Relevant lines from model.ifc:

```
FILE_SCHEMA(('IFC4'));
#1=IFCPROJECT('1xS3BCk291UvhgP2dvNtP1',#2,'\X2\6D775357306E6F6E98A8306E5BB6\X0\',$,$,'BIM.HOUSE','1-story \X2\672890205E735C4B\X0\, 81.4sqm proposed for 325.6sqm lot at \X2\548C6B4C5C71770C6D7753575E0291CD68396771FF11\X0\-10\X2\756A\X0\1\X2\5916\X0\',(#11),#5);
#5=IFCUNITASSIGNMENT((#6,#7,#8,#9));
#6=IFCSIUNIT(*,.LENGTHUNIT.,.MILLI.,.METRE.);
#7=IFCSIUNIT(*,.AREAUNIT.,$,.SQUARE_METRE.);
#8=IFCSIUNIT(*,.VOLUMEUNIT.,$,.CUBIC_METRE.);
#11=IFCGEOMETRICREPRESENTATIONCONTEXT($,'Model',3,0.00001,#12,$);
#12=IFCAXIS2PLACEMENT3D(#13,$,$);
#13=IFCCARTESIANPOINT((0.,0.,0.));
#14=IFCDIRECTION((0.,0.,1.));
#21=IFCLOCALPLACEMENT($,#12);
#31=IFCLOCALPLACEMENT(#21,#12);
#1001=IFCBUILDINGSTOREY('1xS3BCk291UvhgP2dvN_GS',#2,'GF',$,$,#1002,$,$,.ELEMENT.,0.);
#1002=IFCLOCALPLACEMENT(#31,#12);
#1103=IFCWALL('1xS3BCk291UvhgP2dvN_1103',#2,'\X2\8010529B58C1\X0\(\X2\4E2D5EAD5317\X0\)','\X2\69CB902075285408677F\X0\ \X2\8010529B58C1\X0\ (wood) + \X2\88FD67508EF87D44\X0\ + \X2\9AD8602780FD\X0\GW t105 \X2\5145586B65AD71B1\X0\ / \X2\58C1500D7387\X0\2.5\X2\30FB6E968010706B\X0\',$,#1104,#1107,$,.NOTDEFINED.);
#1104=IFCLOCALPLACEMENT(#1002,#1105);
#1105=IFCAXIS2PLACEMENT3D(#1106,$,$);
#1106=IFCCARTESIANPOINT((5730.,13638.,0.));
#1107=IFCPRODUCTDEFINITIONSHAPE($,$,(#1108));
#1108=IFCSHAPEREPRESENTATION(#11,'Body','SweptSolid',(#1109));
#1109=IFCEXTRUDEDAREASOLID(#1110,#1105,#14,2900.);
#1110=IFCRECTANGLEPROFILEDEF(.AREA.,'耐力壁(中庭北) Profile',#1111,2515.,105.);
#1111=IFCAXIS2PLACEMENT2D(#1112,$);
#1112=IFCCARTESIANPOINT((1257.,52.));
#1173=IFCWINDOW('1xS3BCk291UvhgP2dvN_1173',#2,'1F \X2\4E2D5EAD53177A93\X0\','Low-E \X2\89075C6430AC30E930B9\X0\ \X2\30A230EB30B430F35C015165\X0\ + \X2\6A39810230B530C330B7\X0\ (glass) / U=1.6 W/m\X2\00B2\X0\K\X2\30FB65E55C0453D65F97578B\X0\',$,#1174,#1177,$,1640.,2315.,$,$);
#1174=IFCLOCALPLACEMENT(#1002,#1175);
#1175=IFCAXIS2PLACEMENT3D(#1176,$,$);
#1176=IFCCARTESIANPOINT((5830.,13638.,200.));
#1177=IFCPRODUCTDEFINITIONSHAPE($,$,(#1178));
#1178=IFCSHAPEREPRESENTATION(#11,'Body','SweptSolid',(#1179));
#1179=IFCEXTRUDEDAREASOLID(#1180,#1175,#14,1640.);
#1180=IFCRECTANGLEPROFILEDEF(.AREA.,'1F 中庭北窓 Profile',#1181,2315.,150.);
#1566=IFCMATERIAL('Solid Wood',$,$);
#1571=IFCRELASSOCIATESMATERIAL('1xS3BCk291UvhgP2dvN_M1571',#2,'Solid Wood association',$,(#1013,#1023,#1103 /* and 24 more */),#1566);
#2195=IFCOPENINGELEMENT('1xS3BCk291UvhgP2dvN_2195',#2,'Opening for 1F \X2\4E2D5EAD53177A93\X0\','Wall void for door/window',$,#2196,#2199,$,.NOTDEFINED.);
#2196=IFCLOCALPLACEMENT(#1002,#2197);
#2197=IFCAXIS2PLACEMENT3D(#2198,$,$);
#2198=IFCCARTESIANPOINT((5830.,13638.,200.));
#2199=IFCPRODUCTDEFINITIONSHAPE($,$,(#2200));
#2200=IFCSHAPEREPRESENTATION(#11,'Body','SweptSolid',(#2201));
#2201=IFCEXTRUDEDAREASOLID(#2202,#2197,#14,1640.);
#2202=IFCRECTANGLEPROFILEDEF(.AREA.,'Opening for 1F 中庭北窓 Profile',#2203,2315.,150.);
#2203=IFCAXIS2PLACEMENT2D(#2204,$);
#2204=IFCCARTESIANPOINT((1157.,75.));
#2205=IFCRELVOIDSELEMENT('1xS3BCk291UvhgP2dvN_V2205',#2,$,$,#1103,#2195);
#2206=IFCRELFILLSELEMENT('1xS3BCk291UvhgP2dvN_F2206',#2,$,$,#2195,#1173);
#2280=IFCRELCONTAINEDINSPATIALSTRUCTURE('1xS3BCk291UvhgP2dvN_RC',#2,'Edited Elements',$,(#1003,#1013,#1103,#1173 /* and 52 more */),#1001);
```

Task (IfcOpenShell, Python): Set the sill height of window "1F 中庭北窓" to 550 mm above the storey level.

```python
import numpy as np
import ifcopenshell
import ifcopenshell.api.geometry
import ifcopenshell.geom
import ifcopenshell.util.element
import ifcopenshell.util.placement
import ifcopenshell.util.shape
import ifcopenshell.util.unit

model = ifcopenshell.open("model.ifc")
unit_scale = ifcopenshell.util.unit.calculate_unit_scale(model)

window = model.by_guid("1xS3BCk291UvhgP2dvN_1173")
opening = window.FillsVoids[0].RelatingOpeningElement
storey = ifcopenshell.util.element.get_container(window, ifc_class="IfcBuildingStorey")
level = ifcopenshell.util.placement.get_local_placement(storey.ObjectPlacement)[2, 3]

# The opening's origin need not be at the sill, so measure its lowest point.
shape = ifcopenshell.geom.create_shape(ifcopenshell.geom.settings(), opening)
bottom = ifcopenshell.util.shape.get_shape_bottom_elevation(shape, shape.geometry) / unit_scale
dz = level + 0.55 / unit_scale - bottom

shift = np.array([0.0, 0.0, dz])
# The window is not placed relative to its opening, so move both.
for product in (opening, window):
    matrix = ifcopenshell.util.placement.get_local_placement(product.ObjectPlacement)
    matrix[:3, 3] += shift
    ifcopenshell.api.geometry.edit_object_placement(model, product=product, matrix=matrix, is_si=False)

print(f"moved by {dz * unit_scale:+.3f} m")

model.write("model_rev.ifc")
```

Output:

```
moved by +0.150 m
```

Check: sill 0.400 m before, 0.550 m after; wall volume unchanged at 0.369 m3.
